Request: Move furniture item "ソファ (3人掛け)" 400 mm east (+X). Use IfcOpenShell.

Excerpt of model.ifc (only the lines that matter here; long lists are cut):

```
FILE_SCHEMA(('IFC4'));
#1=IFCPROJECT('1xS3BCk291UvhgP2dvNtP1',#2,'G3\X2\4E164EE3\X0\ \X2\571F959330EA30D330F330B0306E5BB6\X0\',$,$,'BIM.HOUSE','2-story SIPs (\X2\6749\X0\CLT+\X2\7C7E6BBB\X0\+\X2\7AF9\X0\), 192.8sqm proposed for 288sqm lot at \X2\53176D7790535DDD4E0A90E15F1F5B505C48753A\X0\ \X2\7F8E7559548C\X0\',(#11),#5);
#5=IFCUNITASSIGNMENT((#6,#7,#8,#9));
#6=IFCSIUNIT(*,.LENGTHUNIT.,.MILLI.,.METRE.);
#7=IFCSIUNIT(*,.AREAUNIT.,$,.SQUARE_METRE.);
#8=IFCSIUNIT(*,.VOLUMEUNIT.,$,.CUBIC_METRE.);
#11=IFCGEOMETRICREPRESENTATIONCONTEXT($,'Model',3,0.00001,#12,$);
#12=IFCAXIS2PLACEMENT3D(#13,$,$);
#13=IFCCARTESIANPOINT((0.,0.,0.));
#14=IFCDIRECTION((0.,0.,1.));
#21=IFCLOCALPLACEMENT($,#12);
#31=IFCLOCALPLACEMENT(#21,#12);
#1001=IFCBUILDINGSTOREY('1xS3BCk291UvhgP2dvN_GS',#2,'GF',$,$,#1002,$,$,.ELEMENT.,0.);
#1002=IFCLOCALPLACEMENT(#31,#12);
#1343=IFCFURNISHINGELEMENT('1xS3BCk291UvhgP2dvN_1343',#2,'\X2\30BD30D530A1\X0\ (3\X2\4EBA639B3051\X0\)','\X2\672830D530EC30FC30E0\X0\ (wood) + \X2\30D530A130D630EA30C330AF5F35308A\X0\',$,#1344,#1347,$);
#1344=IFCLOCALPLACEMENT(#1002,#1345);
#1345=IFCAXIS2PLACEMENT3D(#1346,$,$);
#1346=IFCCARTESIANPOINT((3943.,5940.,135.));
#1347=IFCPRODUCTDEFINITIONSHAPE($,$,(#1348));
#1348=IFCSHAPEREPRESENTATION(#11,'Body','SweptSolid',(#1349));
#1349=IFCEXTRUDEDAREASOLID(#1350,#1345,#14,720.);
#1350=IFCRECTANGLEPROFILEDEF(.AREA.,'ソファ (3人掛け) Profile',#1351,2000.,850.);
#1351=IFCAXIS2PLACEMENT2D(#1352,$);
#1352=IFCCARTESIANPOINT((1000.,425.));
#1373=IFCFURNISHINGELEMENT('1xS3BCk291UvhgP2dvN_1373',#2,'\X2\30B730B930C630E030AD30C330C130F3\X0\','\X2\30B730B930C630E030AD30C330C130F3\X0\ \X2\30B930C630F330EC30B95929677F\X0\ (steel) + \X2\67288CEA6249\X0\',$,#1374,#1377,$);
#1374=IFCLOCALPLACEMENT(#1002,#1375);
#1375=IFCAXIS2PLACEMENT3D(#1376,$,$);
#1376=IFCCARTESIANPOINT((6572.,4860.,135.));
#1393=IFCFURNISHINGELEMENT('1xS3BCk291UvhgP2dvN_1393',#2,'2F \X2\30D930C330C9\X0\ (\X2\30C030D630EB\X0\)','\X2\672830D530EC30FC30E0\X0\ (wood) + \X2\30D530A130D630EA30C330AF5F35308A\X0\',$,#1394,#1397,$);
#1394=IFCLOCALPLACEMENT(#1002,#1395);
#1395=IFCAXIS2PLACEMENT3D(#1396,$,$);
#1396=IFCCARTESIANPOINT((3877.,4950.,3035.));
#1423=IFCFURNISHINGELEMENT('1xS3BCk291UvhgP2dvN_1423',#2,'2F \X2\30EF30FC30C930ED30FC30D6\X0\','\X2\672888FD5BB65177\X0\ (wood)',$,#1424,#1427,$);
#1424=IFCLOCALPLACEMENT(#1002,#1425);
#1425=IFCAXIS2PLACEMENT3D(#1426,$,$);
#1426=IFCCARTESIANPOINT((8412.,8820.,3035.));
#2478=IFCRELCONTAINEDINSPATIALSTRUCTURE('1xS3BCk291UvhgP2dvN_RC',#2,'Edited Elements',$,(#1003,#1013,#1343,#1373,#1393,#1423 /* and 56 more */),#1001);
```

```python
import ifcopenshell
import ifcopenshell.api.geometry
import ifcopenshell.util.placement

model = ifcopenshell.open("model.ifc")

item = model.by_guid("1xS3BCk291UvhgP2dvN_1343")
matrix = ifcopenshell.util.placement.get_local_placement(item.ObjectPlacement)
matrix[0, 3] += 400.0
ifcopenshell.api.geometry.edit_object_placement(model, product=item, matrix=matrix, is_si=False)

print(ifcopenshell.util.placement.get_local_placement(item.ObjectPlacement).round(3) + 0.0)

model.write("model-out.ifc")
```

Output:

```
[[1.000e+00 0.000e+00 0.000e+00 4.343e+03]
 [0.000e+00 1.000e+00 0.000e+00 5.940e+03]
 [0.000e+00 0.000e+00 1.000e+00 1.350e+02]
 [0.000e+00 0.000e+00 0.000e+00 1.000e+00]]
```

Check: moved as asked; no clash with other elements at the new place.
